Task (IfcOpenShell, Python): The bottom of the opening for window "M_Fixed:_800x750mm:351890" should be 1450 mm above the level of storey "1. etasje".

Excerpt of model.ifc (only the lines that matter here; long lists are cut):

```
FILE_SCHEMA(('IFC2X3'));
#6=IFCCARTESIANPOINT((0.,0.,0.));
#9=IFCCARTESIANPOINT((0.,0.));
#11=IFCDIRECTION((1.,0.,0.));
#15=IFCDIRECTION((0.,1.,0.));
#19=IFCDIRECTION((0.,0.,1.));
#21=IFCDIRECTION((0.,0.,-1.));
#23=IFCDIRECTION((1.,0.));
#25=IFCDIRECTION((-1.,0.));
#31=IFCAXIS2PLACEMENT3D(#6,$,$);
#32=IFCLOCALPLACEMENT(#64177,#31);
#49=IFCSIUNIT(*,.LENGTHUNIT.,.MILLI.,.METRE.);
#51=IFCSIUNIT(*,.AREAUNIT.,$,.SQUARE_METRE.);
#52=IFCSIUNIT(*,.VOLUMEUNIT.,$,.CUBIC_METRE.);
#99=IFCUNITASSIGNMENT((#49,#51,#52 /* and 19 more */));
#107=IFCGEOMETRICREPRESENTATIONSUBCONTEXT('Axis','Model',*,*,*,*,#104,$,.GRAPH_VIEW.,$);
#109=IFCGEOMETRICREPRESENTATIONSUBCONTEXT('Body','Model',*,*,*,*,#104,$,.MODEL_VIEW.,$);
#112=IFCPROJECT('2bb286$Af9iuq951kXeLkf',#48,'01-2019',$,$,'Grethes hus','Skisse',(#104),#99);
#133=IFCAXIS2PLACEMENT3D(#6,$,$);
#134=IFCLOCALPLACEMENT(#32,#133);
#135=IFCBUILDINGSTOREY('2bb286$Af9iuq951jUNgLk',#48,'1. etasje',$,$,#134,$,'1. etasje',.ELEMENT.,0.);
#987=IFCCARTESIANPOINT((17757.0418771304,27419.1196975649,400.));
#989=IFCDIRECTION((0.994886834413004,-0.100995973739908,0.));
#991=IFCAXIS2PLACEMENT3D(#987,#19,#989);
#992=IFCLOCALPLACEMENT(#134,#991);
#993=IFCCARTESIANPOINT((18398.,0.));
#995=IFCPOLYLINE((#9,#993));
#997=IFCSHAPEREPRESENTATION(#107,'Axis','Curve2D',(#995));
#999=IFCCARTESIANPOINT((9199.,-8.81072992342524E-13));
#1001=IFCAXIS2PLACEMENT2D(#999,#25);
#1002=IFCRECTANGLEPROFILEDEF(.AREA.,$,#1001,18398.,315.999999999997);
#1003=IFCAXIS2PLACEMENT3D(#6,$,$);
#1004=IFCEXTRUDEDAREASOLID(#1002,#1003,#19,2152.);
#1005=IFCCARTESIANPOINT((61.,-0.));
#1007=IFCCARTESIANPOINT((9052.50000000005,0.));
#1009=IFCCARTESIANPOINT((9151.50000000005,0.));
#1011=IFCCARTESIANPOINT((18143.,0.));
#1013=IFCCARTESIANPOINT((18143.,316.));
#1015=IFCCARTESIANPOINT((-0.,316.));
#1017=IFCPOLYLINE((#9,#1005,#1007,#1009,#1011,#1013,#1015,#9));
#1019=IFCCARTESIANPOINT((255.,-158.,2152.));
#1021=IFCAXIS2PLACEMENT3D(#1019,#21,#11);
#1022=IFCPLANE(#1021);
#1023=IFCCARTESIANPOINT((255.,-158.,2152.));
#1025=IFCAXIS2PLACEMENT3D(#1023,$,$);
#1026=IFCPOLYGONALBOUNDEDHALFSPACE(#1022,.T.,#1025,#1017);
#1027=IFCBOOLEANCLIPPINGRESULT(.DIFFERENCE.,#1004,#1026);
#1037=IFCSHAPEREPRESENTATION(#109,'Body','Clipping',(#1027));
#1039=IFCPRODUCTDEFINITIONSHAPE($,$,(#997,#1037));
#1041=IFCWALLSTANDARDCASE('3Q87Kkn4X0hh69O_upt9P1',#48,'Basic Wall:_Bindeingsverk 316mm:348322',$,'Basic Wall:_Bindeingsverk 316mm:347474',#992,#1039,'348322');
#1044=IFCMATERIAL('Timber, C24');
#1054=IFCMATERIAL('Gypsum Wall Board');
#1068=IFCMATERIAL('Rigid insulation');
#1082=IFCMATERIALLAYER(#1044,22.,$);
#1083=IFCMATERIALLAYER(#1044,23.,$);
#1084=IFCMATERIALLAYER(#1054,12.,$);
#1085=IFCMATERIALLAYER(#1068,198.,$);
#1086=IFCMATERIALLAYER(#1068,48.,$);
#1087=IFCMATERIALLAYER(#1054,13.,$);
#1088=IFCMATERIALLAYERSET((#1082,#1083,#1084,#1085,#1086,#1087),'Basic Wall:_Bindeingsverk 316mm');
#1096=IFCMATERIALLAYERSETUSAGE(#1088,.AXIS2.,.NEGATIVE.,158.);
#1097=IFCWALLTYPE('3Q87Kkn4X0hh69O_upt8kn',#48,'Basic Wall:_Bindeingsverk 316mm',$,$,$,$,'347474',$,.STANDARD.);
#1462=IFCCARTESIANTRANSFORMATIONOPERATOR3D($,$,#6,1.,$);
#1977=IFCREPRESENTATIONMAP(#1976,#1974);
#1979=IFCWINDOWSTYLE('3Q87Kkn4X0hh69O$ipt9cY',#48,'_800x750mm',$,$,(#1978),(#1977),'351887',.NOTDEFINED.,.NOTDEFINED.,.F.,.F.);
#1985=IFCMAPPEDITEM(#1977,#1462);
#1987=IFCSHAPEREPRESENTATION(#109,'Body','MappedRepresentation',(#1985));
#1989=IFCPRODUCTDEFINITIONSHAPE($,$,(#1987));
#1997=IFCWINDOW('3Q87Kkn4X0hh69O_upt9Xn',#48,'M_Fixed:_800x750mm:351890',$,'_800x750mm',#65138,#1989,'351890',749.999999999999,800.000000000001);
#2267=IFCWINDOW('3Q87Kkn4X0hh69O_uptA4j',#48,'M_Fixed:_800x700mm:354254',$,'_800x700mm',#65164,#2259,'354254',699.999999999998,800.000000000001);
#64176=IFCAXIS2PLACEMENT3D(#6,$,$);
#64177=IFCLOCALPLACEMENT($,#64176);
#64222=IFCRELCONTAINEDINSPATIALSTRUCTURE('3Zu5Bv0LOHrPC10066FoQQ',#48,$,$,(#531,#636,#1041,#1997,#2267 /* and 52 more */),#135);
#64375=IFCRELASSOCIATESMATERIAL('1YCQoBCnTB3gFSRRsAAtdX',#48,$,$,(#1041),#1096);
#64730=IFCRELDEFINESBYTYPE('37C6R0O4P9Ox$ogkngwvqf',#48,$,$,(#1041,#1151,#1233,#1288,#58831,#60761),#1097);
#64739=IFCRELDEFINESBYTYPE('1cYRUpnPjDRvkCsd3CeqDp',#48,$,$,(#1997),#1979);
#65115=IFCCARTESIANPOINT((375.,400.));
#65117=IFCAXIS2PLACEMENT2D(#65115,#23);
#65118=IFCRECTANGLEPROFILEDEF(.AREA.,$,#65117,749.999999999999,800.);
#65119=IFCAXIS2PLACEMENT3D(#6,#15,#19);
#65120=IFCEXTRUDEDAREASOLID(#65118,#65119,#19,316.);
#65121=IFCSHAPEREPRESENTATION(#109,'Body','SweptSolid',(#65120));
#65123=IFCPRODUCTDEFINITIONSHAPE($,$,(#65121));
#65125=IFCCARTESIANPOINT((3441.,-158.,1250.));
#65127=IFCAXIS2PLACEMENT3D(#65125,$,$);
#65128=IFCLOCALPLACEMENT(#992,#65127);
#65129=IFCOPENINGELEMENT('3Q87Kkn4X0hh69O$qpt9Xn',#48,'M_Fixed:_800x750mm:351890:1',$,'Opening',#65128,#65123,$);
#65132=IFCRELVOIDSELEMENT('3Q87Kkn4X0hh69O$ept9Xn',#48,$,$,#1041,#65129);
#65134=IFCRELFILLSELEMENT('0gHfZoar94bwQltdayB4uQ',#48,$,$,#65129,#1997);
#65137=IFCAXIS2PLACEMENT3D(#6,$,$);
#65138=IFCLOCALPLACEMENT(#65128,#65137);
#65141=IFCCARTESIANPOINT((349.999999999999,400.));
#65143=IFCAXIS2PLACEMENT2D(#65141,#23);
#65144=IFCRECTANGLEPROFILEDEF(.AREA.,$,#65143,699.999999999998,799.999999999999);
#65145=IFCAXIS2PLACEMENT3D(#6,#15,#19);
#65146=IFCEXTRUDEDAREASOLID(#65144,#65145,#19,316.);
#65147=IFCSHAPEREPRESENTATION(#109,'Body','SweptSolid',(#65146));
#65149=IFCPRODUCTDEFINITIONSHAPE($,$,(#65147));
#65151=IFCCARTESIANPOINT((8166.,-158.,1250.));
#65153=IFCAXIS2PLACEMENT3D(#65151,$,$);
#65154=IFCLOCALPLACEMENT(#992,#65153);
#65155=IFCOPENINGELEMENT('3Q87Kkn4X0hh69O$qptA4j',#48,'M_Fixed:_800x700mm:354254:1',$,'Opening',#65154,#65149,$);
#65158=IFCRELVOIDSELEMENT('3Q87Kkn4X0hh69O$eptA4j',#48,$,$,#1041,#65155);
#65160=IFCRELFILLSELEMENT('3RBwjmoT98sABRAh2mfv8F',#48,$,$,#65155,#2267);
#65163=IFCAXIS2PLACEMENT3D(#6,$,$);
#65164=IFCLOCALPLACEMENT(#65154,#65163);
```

```python
import numpy as np
import ifcopenshell
import ifcopenshell.api.geometry
import ifcopenshell.geom
import ifcopenshell.util.element
import ifcopenshell.util.placement
import ifcopenshell.util.shape
import ifcopenshell.util.unit

model = ifcopenshell.open("model.ifc")
unit_scale = ifcopenshell.util.unit.calculate_unit_scale(model)

window = model.by_guid("3Q87Kkn4X0hh69O_upt9Xn")
opening = window.FillsVoids[0].RelatingOpeningElement
storey = ifcopenshell.util.element.get_container(window, ifc_class="IfcBuildingStorey")
level = ifcopenshell.util.placement.get_local_placement(storey.ObjectPlacement)[2, 3]

# The opening's origin need not be at the sill, so measure its lowest point.
shape = ifcopenshell.geom.create_shape(ifcopenshell.geom.settings(), opening)
bottom = ifcopenshell.util.shape.get_shape_bottom_elevation(shape, shape.geometry) / unit_scale
dz = level + 1450.0 - bottom

shift = np.array([0.0, 0.0, dz])
# The window is placed relative to its opening, so it follows when the opening moves.
matrix = ifcopenshell.util.placement.get_local_placement(opening.ObjectPlacement)
matrix[:3, 3] += shift
ifcopenshell.api.geometry.edit_object_placement(
    model, product=opening, matrix=matrix, is_si=False, should_transform_children=True
)

print(f"moved by {dz * unit_scale:+.3f} m")

model.write("model_rev.ifc")
```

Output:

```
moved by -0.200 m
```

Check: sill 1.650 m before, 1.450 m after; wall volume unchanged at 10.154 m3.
